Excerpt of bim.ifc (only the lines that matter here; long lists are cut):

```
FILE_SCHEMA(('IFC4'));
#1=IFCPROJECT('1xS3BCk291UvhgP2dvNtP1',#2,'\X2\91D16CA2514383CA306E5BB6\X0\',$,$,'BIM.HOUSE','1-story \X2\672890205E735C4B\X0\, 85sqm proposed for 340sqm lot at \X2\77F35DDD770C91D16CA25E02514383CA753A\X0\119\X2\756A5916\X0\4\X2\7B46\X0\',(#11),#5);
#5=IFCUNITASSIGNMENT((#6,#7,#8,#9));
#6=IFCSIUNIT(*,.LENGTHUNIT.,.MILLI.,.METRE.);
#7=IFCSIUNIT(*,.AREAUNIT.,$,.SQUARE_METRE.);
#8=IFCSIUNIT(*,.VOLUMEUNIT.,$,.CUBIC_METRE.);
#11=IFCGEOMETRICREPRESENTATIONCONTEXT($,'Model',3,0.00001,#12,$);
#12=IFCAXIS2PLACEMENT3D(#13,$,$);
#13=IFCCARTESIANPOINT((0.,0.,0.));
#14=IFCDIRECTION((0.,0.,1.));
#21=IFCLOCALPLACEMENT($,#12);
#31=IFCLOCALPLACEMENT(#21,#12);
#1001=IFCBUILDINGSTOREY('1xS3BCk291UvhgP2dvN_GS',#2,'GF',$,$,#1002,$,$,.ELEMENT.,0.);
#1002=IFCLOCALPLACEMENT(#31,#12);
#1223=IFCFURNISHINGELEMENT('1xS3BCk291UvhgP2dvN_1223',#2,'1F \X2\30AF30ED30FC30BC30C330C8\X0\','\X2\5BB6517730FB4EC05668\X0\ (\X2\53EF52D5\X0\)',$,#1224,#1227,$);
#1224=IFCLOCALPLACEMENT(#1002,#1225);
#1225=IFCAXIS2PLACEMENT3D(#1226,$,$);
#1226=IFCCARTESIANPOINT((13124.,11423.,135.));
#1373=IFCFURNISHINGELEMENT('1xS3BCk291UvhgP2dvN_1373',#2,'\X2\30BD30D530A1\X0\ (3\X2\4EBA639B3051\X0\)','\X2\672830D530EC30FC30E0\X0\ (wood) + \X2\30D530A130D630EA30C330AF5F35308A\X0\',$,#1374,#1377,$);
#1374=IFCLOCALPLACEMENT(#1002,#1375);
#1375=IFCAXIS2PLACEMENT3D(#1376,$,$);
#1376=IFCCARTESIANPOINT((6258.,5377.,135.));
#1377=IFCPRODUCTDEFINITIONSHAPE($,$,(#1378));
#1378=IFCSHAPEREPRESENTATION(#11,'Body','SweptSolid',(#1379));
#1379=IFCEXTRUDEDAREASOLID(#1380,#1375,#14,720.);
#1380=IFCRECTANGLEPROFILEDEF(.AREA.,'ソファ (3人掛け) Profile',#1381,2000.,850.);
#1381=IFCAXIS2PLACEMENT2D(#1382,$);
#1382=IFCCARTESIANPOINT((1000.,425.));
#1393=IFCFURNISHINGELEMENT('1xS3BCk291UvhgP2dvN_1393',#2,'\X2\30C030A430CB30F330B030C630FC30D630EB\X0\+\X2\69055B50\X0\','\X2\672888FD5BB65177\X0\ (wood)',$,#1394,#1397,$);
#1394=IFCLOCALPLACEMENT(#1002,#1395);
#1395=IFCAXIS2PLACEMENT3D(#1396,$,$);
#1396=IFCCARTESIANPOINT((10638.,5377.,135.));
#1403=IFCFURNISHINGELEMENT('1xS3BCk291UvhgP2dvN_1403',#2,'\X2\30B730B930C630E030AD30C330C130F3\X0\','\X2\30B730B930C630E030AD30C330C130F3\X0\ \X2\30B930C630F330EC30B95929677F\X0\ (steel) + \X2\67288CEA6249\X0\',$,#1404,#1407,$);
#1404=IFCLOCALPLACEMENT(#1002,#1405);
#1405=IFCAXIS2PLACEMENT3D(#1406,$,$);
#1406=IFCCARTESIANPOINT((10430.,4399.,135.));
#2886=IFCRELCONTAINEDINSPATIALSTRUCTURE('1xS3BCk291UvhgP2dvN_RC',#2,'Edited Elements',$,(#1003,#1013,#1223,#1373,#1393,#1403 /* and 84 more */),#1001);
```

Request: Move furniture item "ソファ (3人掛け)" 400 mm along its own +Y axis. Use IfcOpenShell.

```python
import ifcopenshell
import ifcopenshell.api.geometry
import ifcopenshell.util.placement
import ifcopenshell.util.unit

model = ifcopenshell.open("bim.ifc")
unit_scale = ifcopenshell.util.unit.calculate_unit_scale(model)

item = model.by_id(1373)
matrix = ifcopenshell.util.placement.get_local_placement(item.ObjectPlacement)
matrix[:3, 3] += matrix[:3, 1] * 0.4 / unit_scale
ifcopenshell.api.geometry.edit_object_placement(model, product=item, matrix=matrix, is_si=False)

print(ifcopenshell.util.placement.get_local_placement(item.ObjectPlacement).round(3) + 0.0)

model.write("bim_edited.ifc")
```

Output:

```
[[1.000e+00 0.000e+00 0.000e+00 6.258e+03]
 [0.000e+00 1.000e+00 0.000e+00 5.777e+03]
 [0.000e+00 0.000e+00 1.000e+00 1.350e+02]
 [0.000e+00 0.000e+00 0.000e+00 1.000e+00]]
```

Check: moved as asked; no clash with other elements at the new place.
